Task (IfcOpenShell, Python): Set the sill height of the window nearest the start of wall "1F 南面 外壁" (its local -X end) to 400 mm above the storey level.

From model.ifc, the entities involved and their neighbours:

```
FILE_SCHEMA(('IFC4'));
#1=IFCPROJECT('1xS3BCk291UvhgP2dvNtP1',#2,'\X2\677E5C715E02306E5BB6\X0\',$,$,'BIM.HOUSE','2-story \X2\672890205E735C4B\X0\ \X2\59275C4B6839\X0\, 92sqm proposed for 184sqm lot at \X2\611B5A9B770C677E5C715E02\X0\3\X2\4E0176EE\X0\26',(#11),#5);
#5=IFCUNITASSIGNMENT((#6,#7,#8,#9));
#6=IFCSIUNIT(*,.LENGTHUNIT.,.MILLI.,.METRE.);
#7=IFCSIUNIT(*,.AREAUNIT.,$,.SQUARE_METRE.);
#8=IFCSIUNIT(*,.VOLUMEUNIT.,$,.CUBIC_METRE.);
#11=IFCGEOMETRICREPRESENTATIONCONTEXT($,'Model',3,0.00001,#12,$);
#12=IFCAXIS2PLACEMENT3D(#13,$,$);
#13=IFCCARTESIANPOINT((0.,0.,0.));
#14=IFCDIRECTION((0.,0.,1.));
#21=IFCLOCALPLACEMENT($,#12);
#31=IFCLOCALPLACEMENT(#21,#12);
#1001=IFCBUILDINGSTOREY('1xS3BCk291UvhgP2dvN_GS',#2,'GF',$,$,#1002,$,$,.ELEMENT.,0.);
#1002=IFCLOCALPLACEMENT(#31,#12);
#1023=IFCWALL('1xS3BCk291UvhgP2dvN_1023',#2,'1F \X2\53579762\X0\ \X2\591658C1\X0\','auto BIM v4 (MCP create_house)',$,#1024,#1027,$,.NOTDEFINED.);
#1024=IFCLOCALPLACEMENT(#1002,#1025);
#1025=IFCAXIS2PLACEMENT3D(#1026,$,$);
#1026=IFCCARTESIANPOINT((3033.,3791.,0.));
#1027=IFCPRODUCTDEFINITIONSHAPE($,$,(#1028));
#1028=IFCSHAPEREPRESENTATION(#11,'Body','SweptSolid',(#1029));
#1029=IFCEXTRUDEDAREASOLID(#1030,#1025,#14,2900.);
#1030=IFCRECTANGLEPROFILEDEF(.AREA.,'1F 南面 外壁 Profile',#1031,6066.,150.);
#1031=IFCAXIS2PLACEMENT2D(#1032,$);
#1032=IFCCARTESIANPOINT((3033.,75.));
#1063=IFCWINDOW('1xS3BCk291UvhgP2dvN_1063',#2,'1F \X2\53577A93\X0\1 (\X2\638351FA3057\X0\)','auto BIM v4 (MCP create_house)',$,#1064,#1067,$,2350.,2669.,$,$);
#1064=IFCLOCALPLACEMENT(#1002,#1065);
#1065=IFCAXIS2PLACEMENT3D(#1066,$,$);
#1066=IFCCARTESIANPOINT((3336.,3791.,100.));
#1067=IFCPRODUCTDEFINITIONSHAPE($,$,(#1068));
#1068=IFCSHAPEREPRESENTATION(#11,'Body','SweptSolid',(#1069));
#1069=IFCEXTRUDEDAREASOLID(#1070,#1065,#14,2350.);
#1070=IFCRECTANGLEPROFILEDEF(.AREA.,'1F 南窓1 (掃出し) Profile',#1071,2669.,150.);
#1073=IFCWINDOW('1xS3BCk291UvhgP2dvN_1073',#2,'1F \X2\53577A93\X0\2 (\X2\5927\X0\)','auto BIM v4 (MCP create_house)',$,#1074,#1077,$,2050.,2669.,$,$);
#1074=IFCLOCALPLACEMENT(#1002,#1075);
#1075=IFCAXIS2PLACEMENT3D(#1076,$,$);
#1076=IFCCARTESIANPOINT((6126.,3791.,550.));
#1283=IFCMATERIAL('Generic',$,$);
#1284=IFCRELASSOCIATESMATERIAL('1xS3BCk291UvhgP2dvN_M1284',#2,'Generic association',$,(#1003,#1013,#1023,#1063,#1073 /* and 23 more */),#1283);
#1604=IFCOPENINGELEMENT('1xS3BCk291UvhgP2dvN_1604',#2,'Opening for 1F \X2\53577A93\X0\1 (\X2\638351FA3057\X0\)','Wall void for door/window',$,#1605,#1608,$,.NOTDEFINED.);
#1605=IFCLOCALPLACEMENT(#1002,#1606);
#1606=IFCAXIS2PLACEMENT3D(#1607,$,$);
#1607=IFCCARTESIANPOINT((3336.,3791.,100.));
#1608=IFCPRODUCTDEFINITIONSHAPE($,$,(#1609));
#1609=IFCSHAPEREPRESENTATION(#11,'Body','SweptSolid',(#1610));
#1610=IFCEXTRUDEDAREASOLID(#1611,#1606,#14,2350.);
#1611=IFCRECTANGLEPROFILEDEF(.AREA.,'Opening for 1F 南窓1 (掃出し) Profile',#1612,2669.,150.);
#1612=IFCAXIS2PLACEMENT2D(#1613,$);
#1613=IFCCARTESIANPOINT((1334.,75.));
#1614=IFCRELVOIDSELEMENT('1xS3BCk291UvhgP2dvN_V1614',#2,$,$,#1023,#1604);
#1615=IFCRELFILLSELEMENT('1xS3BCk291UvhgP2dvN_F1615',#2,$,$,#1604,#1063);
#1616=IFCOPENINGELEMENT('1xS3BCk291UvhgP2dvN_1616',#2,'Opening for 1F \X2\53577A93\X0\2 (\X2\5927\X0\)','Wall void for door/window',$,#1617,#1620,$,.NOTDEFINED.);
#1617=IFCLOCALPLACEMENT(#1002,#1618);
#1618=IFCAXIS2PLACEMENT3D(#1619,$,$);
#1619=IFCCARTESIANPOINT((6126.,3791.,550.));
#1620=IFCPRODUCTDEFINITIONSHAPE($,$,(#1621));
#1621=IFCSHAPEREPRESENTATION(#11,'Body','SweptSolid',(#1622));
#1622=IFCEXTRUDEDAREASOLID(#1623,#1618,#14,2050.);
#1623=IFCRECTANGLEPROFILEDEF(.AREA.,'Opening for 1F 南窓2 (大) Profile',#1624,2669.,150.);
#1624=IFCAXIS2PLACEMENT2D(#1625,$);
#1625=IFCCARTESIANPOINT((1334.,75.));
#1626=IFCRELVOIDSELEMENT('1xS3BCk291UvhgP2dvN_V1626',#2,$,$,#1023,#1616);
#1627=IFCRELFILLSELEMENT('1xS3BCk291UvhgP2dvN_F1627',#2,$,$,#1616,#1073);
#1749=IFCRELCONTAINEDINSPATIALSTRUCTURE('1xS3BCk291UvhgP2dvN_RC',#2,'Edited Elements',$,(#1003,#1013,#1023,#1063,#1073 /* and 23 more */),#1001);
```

```python
import numpy as np
import ifcopenshell
import ifcopenshell.api.geometry
import ifcopenshell.geom
import ifcopenshell.util.element
import ifcopenshell.util.placement
import ifcopenshell.util.shape
import ifcopenshell.util.unit

model = ifcopenshell.open("model.ifc")
unit_scale = ifcopenshell.util.unit.calculate_unit_scale(model)

window = model.by_guid("1xS3BCk291UvhgP2dvN_1063")
opening = window.FillsVoids[0].RelatingOpeningElement
storey = ifcopenshell.util.element.get_container(window, ifc_class="IfcBuildingStorey")
level = ifcopenshell.util.placement.get_local_placement(storey.ObjectPlacement)[2, 3]

# The opening's origin need not be at the sill, so measure its lowest point.
shape = ifcopenshell.geom.create_shape(ifcopenshell.geom.settings(), opening)
bottom = ifcopenshell.util.shape.get_shape_bottom_elevation(shape, shape.geometry) / unit_scale
dz = level + 0.4 / unit_scale - bottom

shift = np.array([0.0, 0.0, dz])
# The window is not placed relative to its opening, so move both.
for product in (opening, window):
    matrix = ifcopenshell.util.placement.get_local_placement(product.ObjectPlacement)
    matrix[:3, 3] += shift
    ifcopenshell.api.geometry.edit_object_placement(model, product=product, matrix=matrix, is_si=False)

print(f"moved by {dz * unit_scale:+.3f} m")

model.write("model_edited.ifc")
```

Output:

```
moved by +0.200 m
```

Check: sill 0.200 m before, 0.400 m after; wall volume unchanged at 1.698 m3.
